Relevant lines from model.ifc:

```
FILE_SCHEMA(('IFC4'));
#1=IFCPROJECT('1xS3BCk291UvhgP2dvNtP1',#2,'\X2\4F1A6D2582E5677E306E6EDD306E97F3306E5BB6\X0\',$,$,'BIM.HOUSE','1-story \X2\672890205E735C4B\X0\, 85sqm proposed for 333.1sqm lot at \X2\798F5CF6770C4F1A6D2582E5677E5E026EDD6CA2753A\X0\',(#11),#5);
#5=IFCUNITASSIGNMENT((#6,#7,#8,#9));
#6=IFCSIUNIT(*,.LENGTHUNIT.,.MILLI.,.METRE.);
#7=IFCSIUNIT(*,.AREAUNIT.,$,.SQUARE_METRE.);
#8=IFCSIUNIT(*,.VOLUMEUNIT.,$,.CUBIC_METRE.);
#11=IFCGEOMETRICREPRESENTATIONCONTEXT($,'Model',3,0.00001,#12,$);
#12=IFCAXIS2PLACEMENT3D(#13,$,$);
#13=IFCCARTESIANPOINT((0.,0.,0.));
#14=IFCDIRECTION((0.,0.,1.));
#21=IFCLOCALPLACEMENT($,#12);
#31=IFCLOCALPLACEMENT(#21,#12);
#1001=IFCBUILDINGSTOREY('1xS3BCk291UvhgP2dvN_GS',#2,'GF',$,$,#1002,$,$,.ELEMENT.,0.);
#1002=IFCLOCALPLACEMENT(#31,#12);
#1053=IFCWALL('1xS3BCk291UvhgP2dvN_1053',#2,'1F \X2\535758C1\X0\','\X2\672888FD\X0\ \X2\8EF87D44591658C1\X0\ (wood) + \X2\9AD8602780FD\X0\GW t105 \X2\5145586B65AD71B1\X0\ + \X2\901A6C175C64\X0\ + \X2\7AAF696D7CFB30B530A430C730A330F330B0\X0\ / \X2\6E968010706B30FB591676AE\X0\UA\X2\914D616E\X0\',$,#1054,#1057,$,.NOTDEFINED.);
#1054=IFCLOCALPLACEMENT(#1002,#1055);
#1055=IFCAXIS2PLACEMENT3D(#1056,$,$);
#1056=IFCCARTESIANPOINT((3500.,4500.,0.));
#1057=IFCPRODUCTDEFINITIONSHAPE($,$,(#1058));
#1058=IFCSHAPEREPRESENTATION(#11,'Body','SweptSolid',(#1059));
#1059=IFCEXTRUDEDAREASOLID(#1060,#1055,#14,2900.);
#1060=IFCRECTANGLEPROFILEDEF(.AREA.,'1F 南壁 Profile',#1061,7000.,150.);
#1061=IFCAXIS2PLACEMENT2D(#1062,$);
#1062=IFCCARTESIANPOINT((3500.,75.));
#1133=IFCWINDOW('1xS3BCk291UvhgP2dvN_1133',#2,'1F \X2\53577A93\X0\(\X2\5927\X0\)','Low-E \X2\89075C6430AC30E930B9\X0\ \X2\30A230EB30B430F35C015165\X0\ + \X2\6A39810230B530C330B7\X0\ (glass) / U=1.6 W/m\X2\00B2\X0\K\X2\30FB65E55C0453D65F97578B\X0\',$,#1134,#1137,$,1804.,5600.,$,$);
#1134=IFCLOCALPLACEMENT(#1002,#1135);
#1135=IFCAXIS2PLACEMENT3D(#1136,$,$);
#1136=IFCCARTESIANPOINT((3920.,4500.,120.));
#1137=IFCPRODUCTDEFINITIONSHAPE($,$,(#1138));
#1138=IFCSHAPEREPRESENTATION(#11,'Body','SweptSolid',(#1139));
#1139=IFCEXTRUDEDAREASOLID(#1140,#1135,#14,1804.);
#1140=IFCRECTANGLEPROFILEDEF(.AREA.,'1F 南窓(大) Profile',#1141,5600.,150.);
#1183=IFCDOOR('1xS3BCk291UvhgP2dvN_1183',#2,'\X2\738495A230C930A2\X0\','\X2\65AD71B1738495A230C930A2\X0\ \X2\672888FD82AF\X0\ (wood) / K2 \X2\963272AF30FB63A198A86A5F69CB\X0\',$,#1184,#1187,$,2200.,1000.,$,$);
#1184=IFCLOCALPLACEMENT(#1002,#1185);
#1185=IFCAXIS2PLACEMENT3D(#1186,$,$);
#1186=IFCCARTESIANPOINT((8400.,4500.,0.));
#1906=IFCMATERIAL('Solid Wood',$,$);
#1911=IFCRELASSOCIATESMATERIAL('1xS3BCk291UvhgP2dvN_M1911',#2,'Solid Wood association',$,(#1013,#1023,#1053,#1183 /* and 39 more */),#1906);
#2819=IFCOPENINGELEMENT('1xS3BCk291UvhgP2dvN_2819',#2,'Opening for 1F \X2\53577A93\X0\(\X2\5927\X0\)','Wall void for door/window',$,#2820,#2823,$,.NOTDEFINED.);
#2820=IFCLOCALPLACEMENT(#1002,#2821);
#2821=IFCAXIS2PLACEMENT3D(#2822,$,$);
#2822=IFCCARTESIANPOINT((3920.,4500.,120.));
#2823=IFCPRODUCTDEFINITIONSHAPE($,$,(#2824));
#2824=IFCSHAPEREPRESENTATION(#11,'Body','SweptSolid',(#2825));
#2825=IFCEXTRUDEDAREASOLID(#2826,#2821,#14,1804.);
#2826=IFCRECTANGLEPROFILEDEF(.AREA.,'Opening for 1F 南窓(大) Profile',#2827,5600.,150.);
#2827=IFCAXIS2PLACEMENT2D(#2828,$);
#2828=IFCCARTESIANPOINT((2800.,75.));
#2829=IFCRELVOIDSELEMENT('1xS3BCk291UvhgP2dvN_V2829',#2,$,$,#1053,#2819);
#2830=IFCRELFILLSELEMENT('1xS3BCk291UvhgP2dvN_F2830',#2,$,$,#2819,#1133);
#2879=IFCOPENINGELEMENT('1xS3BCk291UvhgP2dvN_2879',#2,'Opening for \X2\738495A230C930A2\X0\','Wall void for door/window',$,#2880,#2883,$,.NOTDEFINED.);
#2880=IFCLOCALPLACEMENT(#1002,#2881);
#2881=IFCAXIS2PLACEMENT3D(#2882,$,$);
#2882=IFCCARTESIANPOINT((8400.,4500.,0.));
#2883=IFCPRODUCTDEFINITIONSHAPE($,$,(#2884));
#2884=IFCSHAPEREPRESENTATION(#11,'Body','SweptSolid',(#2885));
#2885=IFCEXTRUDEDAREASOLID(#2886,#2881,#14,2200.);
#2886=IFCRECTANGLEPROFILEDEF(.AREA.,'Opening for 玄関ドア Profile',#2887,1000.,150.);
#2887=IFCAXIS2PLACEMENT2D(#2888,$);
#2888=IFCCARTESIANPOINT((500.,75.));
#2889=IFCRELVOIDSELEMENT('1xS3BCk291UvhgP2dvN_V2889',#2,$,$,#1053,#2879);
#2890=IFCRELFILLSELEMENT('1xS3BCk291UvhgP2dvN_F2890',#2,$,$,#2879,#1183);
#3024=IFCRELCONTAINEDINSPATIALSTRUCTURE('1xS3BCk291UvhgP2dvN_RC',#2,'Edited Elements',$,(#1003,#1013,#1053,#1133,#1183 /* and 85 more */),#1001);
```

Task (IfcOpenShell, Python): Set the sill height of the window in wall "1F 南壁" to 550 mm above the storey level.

```python
import numpy as np
import ifcopenshell
import ifcopenshell.api.geometry
import ifcopenshell.geom
import ifcopenshell.util.element
import ifcopenshell.util.placement
import ifcopenshell.util.shape
import ifcopenshell.util.unit

model = ifcopenshell.open("model.ifc")
unit_scale = ifcopenshell.util.unit.calculate_unit_scale(model)

window = model.by_guid("1xS3BCk291UvhgP2dvN_1133")
opening = window.FillsVoids[0].RelatingOpeningElement
storey = ifcopenshell.util.element.get_container(window, ifc_class="IfcBuildingStorey")
level = ifcopenshell.util.placement.get_local_placement(storey.ObjectPlacement)[2, 3]

# The opening's origin need not be at the sill, so measure its lowest point.
shape = ifcopenshell.geom.create_shape(ifcopenshell.geom.settings(), opening)
bottom = ifcopenshell.util.shape.get_shape_bottom_elevation(shape, shape.geometry) / unit_scale
dz = level + 0.55 / unit_scale - bottom

shift = np.array([0.0, 0.0, dz])
# The window is not placed relative to its opening, so move both.
for product in (opening, window):
    matrix = ifcopenshell.util.placement.get_local_placement(product.ObjectPlacement)
    matrix[:3, 3] += shift
    ifcopenshell.api.geometry.edit_object_placement(model, product=product, matrix=matrix, is_si=False)

print(f"moved by {dz * unit_scale:+.3f} m")

model.write("model_rev.ifc")
```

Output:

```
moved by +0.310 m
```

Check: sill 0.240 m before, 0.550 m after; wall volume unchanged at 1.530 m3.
